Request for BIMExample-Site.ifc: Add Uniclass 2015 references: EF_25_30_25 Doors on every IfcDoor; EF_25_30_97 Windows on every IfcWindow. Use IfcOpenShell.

First a look at what the model holds.

```python
import ifcopenshell

model = ifcopenshell.open("BIMExample-Site.ifc")
print(model.schema)
print("classifications:", [c.Name for c in model.by_type("IfcClassification")])
for ifc_class in ("IfcDoor", "IfcRoof", "IfcStair", "IfcWall", "IfcWindow"):
    print(ifc_class, len(model.by_type(ifc_class)))
```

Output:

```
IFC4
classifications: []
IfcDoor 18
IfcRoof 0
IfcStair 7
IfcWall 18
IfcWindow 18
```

```python
import ifcopenshell
import ifcopenshell.api.classification

model = ifcopenshell.open("BIMExample-Site.ifc")

system = ifcopenshell.api.classification.add_classification(model, classification="Uniclass 2015")

codes = {
    "IfcDoor": ("EF_25_30_25", "Doors"),
    "IfcWindow": ("EF_25_30_97", "Windows"),
}
for ifc_class, (code, name) in codes.items():
    products = model.by_type(ifc_class)
    ifcopenshell.api.classification.add_reference(
        model, products=products, classification=system, identification=code, name=name
    )
    print(code, len(products))

model.write("BIMExample-Site_rev.ifc")
```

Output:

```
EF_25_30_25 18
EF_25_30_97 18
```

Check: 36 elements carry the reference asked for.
